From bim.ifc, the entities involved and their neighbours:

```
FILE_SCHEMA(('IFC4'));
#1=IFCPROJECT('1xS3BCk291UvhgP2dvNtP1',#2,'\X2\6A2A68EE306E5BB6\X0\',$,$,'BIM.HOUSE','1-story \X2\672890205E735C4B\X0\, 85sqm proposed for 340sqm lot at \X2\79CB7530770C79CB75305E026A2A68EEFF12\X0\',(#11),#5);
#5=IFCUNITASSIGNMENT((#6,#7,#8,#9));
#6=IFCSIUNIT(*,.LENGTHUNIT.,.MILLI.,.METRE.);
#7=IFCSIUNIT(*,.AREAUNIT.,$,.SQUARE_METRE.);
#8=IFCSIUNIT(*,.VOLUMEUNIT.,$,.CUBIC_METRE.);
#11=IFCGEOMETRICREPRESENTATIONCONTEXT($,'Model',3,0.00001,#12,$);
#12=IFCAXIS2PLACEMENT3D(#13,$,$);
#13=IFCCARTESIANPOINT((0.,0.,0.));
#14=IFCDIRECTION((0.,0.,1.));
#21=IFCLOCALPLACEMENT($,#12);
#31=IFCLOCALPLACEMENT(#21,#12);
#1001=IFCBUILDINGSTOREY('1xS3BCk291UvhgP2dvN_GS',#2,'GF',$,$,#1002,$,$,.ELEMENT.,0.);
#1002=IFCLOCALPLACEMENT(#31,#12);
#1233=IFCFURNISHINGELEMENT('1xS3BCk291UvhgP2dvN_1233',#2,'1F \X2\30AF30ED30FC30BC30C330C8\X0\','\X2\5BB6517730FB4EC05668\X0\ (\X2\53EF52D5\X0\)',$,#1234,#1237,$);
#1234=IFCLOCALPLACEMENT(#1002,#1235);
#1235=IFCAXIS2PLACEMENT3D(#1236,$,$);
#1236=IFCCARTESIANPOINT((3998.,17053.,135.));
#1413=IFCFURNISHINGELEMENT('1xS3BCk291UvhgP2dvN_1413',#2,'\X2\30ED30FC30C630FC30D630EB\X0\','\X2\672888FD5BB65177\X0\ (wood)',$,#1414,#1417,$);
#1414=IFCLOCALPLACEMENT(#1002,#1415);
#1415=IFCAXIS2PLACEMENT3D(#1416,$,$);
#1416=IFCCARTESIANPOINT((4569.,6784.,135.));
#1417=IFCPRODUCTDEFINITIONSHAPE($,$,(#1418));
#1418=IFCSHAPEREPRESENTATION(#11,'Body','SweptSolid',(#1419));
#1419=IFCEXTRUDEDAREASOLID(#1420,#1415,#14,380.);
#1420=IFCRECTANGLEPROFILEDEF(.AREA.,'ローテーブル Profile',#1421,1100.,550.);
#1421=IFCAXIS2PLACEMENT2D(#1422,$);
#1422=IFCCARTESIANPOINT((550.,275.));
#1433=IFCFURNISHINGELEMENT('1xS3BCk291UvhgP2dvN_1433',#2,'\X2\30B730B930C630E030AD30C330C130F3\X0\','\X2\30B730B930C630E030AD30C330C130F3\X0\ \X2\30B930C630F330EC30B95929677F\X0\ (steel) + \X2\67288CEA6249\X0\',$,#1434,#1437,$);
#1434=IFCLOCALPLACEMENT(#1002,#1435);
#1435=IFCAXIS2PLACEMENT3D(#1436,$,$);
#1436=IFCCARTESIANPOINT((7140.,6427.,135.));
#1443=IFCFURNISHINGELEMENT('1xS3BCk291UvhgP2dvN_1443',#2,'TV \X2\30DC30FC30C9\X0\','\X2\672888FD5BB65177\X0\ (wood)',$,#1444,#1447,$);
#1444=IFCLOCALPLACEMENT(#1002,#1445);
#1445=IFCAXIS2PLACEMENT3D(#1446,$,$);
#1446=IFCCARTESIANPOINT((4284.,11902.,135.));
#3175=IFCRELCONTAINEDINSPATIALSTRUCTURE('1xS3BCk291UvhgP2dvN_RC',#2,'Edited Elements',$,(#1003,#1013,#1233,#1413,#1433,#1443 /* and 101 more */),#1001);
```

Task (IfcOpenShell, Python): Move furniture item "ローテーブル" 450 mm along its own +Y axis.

```python
import ifcopenshell
import ifcopenshell.api.geometry
import ifcopenshell.util.placement
import ifcopenshell.util.unit

model = ifcopenshell.open("bim.ifc")
unit_scale = ifcopenshell.util.unit.calculate_unit_scale(model)

item = model.by_guid("1xS3BCk291UvhgP2dvN_1413")
matrix = ifcopenshell.util.placement.get_local_placement(item.ObjectPlacement)
matrix[:3, 3] += matrix[:3, 1] * 0.45 / unit_scale
ifcopenshell.api.geometry.edit_object_placement(model, product=item, matrix=matrix, is_si=False)

print(ifcopenshell.util.placement.get_local_placement(item.ObjectPlacement).round(3) + 0.0)

model.write("bim_v2.ifc")
```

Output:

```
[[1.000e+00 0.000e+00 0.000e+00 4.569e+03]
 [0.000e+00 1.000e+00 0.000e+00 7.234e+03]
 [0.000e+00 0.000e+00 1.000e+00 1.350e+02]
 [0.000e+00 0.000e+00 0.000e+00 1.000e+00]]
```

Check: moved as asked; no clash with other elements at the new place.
